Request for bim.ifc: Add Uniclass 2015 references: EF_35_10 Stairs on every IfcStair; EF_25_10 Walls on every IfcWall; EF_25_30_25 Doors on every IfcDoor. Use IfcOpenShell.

First a look at what the model holds.

```python
import ifcopenshell

model = ifcopenshell.open("bim.ifc")
print(model.schema)
print("classifications:", [c.Name for c in model.by_type("IfcClassification")])
for ifc_class in ("IfcDoor", "IfcRoof", "IfcStair", "IfcWall", "IfcWindow"):
    print(ifc_class, len(model.by_type(ifc_class)))
```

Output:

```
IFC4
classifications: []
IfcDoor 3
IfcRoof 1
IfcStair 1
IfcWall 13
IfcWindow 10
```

```python
import ifcopenshell
import ifcopenshell.api.classification

model = ifcopenshell.open("bim.ifc")

system = ifcopenshell.api.classification.add_classification(model, classification="Uniclass 2015")

codes = {
    "IfcStair": ("EF_35_10", "Stairs"),
    "IfcWall": ("EF_25_10", "Walls"),
    "IfcDoor": ("EF_25_30_25", "Doors"),
}
for ifc_class, (code, name) in codes.items():
    products = model.by_type(ifc_class)
    ifcopenshell.api.classification.add_reference(
        model, products=products, classification=system, identification=code, name=name
    )
    print(code, len(products))

model.write("bim_updated.ifc")
```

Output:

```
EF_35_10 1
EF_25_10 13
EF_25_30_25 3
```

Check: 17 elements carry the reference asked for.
